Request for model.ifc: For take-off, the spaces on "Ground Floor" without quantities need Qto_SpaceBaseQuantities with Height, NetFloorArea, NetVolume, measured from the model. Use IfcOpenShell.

First a look at what the model holds.

```python
import ifcopenshell
import ifcopenshell.util.element
import ifcopenshell.util.unit

model = ifcopenshell.open("model.ifc")
print(model.schema)
for unit_type in ("LENGTHUNIT", "AREAUNIT", "VOLUMEUNIT"):
    print(unit_type, ifcopenshell.util.unit.calculate_unit_scale(model, unit_type))
storey = next(s for s in model.by_type("IfcBuildingStorey") if s.Name == "Ground Floor")
spaces = [e for e in ifcopenshell.util.element.get_decomposition(storey) if e.is_a("IfcSpace")]
for e in sorted(spaces, key=lambda e: e.id()):
    print(e.id(), e.is_a(), e.Name, list(ifcopenshell.util.element.get_psets(e, qtos_only=True)), sep=" | ")
```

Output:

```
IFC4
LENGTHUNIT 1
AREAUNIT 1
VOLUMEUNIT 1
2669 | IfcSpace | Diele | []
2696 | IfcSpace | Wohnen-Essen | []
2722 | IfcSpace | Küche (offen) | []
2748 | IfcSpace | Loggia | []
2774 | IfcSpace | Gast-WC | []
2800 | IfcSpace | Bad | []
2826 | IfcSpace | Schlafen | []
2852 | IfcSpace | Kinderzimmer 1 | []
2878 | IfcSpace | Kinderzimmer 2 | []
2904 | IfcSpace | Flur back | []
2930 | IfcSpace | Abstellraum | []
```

```python
import ifcopenshell
import ifcopenshell.api.pset
import ifcopenshell.geom
import ifcopenshell.util.element
import ifcopenshell.util.shape
import ifcopenshell.util.unit

model = ifcopenshell.open("model.ifc")
unit_scale = ifcopenshell.util.unit.calculate_unit_scale(model)
area_scale = ifcopenshell.util.unit.calculate_unit_scale(model, "AREAUNIT")
volume_scale = ifcopenshell.util.unit.calculate_unit_scale(model, "VOLUMEUNIT")
settings = ifcopenshell.geom.settings()

storey = next(s for s in model.by_type("IfcBuildingStorey") if s.Name == "Ground Floor")
spaces = [e for e in ifcopenshell.util.element.get_decomposition(storey) if e.is_a("IfcSpace")]

for e in sorted(spaces, key=lambda e: e.id()):
    if ifcopenshell.util.element.get_psets(e, qtos_only=True, should_inherit=False):
        continue
    # Geometry comes back in metres, in the element's own axes.
    shape = ifcopenshell.geom.create_shape(settings, e)
    values = {
        "Height": ifcopenshell.util.shape.get_z(shape.geometry) / unit_scale,
        "NetFloorArea": ifcopenshell.util.shape.get_footprint_area(shape.geometry) / area_scale,
        "NetVolume": ifcopenshell.util.shape.get_volume(shape.geometry) / volume_scale,
    }
    qto = ifcopenshell.api.pset.add_qto(model, product=e, name="Qto_SpaceBaseQuantities")
    ifcopenshell.api.pset.edit_qto(model, qto=qto, properties=values)
    print(e.id(), {k: round(v, 3) for k, v in values.items()})

model.write("model-out.ifc")
```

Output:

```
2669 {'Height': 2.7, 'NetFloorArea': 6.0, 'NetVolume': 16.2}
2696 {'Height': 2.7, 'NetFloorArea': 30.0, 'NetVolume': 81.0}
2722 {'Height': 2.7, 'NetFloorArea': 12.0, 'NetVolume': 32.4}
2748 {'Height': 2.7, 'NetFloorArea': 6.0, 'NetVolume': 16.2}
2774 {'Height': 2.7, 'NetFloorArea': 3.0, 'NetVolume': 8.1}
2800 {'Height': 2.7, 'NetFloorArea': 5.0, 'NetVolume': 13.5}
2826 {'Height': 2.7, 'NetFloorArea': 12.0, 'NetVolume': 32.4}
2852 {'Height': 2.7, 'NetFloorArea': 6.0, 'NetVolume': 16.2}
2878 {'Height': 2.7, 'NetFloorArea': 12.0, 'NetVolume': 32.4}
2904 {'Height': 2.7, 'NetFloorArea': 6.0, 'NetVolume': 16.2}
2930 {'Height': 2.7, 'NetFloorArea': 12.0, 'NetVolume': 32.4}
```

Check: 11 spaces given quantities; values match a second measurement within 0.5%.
